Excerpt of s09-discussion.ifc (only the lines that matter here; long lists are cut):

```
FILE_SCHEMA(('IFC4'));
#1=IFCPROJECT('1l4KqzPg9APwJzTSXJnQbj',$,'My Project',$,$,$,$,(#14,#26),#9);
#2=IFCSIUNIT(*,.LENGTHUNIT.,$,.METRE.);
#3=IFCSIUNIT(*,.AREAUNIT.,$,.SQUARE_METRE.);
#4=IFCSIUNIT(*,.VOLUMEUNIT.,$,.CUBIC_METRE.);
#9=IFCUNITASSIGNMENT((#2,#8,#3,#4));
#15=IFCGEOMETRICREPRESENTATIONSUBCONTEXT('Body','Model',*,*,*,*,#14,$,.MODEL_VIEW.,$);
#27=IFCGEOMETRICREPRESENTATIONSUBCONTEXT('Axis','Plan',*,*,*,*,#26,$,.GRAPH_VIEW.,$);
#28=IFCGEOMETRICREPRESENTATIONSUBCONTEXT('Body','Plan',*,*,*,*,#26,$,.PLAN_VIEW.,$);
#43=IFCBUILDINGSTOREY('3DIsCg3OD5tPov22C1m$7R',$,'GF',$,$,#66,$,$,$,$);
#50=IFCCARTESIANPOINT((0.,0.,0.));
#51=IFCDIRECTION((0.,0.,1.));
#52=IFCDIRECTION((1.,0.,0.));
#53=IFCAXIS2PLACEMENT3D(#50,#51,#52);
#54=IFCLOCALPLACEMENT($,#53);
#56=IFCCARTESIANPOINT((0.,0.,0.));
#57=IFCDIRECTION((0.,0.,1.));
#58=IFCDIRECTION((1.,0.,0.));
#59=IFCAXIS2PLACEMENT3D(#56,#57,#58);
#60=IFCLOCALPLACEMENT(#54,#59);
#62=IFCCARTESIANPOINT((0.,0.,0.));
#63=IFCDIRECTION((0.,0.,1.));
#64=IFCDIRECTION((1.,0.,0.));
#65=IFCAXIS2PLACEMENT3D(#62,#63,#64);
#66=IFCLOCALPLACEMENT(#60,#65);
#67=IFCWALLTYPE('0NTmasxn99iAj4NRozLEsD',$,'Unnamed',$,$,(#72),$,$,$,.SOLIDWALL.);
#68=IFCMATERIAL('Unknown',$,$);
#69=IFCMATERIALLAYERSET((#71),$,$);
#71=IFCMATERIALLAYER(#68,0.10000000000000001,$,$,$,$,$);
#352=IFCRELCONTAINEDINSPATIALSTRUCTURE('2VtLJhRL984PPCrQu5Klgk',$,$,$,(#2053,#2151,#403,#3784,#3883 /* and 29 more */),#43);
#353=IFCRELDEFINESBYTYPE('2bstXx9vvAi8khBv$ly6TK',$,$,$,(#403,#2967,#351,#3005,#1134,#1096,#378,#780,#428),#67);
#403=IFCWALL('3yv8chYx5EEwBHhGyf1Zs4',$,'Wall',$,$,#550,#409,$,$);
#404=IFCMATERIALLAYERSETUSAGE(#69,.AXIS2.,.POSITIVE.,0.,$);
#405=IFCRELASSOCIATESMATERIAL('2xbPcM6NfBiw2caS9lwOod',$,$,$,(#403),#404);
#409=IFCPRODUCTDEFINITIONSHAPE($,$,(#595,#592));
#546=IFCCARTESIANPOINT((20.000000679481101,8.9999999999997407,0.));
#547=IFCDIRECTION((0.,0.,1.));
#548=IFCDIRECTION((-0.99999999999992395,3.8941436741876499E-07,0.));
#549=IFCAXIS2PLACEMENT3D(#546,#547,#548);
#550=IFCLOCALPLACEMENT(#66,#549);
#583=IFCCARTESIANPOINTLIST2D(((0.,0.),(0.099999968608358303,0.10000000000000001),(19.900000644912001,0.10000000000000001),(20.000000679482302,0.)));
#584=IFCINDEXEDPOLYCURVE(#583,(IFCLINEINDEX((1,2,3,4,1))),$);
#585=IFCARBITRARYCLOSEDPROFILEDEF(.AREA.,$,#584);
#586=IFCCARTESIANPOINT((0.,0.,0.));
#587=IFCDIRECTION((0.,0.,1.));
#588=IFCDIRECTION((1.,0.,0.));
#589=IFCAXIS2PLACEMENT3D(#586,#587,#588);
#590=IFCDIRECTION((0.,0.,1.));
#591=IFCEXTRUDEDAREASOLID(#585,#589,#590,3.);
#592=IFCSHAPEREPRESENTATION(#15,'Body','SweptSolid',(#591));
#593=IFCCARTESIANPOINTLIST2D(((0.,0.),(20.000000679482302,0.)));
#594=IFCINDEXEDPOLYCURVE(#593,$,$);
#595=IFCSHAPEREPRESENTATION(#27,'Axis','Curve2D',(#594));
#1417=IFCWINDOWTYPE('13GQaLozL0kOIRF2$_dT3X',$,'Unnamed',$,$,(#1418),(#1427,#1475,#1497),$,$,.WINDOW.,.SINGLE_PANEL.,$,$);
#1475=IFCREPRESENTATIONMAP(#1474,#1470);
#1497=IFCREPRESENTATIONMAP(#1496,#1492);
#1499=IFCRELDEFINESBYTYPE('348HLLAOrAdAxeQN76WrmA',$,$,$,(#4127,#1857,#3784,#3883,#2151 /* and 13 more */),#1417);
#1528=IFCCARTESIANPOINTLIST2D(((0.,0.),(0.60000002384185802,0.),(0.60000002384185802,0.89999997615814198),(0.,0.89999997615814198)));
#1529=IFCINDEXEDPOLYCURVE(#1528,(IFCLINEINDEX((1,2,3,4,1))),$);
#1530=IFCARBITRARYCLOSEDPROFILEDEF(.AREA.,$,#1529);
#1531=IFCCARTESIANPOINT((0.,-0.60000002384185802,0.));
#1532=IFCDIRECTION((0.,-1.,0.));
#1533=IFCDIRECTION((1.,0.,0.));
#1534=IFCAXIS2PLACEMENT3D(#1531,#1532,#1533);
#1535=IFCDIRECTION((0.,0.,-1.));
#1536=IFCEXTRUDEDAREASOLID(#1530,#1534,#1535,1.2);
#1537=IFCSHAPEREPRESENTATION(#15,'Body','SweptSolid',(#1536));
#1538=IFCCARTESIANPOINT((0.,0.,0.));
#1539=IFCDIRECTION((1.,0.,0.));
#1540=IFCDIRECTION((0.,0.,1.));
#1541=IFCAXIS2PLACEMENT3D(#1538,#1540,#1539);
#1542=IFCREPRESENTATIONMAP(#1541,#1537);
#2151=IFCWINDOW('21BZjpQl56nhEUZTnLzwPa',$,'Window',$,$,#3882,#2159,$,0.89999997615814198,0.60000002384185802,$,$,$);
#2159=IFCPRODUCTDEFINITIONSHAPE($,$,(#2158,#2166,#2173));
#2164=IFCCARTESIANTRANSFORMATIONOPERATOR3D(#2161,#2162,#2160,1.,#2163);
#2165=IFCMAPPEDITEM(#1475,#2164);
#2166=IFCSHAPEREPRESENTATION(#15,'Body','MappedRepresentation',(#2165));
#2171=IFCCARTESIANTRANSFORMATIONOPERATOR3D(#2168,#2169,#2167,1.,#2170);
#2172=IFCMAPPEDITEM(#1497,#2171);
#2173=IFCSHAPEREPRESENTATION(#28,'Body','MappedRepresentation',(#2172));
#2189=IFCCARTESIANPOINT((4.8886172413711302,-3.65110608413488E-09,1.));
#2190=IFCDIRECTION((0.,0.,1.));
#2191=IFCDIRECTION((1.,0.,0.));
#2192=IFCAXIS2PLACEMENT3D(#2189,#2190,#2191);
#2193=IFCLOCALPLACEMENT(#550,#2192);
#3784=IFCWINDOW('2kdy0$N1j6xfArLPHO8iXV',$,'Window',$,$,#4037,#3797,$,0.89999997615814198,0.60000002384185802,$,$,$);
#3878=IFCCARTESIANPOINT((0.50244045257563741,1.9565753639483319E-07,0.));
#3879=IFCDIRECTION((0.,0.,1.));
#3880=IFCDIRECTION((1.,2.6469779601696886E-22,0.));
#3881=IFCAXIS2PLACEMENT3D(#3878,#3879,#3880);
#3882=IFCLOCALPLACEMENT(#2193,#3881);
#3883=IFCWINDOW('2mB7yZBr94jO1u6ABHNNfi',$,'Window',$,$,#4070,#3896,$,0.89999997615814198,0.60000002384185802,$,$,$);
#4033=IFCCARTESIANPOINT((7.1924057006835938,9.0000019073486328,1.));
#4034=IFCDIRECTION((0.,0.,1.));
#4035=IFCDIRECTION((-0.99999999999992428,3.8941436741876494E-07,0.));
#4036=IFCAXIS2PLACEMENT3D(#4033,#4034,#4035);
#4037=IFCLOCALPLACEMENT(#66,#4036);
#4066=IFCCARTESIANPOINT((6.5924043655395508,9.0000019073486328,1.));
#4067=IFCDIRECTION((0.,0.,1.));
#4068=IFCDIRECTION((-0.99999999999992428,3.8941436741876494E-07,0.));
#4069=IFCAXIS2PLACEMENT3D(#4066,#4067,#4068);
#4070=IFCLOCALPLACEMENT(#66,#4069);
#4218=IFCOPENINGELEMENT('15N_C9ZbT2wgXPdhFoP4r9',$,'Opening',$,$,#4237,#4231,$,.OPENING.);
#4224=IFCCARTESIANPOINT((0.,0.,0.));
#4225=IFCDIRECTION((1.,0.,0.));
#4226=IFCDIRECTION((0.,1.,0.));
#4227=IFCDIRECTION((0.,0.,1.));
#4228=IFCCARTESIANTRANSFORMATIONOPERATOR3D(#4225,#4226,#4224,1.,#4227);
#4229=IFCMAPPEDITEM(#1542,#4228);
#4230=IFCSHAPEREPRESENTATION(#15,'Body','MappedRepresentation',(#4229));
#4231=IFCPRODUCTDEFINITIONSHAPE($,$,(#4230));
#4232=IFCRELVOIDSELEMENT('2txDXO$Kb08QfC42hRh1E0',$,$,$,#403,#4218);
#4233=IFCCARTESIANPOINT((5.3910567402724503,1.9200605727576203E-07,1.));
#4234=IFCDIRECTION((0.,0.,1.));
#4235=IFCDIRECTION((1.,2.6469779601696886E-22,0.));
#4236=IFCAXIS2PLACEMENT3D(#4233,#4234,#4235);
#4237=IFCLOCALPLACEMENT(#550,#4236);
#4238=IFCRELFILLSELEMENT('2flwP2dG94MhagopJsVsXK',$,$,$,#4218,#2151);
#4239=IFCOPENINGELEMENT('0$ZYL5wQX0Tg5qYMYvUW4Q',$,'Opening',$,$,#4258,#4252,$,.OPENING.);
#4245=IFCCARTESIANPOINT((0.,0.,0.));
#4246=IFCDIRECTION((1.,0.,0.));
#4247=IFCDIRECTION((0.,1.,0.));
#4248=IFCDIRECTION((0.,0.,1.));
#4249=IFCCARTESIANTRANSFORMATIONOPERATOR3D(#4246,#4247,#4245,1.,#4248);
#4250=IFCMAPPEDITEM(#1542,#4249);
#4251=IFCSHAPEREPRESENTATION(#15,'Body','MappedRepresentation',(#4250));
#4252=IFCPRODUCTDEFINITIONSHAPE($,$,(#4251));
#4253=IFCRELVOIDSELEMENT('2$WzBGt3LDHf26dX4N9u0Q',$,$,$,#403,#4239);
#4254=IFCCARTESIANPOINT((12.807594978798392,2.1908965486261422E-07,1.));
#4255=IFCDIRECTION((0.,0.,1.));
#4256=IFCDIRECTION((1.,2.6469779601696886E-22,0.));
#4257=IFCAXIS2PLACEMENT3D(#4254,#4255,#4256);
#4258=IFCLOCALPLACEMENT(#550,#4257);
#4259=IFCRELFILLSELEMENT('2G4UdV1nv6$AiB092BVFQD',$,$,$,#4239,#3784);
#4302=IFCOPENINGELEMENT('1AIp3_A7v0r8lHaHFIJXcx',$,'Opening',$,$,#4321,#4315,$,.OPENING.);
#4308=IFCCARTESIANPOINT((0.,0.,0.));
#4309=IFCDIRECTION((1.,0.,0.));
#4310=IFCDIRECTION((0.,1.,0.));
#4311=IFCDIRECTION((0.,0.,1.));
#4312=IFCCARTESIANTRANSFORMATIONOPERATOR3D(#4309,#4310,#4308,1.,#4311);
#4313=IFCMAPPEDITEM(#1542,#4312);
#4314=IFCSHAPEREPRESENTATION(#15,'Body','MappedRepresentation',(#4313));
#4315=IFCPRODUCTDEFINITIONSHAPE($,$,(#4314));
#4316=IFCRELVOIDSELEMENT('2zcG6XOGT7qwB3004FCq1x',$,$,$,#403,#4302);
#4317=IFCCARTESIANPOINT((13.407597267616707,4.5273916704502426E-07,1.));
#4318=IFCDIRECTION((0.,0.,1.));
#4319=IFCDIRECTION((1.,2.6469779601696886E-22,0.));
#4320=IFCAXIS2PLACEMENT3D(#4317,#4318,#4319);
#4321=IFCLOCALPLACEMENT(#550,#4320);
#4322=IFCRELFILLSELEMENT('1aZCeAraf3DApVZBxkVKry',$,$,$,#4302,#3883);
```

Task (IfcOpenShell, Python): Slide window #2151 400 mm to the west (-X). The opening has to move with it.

```python
import ifcopenshell
import ifcopenshell.api.geometry
import ifcopenshell.util.placement
import ifcopenshell.util.unit

model = ifcopenshell.open("s09-discussion.ifc")
unit_scale = ifcopenshell.util.unit.calculate_unit_scale(model)

window = model.by_guid("21BZjpQl56nhEUZTnLzwPa")
opening = window.FillsVoids[0].RelatingOpeningElement
wall = opening.VoidsElements[0].RelatingBuildingElement

wall_matrix = ifcopenshell.util.placement.get_local_placement(wall.ObjectPlacement)
shift = wall_matrix[:3, 0] * 0.4 / unit_scale
before = ifcopenshell.util.placement.get_local_placement(window.ObjectPlacement)[:3, 3].copy()

# The window is not placed relative to its opening, so move both.
for product in (opening, window):
    matrix = ifcopenshell.util.placement.get_local_placement(product.ObjectPlacement)
    matrix[:3, 3] += shift
    ifcopenshell.api.geometry.edit_object_placement(model, product=product, matrix=matrix, is_si=False)

after = ifcopenshell.util.placement.get_local_placement(window.ObjectPlacement)[:3, 3]
print("window moved by", (after - before).round(3) + 0.0)

model.write("s09-discussion_updated.ifc")
```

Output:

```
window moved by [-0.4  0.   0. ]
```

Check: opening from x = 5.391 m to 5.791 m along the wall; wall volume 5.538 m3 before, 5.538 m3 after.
